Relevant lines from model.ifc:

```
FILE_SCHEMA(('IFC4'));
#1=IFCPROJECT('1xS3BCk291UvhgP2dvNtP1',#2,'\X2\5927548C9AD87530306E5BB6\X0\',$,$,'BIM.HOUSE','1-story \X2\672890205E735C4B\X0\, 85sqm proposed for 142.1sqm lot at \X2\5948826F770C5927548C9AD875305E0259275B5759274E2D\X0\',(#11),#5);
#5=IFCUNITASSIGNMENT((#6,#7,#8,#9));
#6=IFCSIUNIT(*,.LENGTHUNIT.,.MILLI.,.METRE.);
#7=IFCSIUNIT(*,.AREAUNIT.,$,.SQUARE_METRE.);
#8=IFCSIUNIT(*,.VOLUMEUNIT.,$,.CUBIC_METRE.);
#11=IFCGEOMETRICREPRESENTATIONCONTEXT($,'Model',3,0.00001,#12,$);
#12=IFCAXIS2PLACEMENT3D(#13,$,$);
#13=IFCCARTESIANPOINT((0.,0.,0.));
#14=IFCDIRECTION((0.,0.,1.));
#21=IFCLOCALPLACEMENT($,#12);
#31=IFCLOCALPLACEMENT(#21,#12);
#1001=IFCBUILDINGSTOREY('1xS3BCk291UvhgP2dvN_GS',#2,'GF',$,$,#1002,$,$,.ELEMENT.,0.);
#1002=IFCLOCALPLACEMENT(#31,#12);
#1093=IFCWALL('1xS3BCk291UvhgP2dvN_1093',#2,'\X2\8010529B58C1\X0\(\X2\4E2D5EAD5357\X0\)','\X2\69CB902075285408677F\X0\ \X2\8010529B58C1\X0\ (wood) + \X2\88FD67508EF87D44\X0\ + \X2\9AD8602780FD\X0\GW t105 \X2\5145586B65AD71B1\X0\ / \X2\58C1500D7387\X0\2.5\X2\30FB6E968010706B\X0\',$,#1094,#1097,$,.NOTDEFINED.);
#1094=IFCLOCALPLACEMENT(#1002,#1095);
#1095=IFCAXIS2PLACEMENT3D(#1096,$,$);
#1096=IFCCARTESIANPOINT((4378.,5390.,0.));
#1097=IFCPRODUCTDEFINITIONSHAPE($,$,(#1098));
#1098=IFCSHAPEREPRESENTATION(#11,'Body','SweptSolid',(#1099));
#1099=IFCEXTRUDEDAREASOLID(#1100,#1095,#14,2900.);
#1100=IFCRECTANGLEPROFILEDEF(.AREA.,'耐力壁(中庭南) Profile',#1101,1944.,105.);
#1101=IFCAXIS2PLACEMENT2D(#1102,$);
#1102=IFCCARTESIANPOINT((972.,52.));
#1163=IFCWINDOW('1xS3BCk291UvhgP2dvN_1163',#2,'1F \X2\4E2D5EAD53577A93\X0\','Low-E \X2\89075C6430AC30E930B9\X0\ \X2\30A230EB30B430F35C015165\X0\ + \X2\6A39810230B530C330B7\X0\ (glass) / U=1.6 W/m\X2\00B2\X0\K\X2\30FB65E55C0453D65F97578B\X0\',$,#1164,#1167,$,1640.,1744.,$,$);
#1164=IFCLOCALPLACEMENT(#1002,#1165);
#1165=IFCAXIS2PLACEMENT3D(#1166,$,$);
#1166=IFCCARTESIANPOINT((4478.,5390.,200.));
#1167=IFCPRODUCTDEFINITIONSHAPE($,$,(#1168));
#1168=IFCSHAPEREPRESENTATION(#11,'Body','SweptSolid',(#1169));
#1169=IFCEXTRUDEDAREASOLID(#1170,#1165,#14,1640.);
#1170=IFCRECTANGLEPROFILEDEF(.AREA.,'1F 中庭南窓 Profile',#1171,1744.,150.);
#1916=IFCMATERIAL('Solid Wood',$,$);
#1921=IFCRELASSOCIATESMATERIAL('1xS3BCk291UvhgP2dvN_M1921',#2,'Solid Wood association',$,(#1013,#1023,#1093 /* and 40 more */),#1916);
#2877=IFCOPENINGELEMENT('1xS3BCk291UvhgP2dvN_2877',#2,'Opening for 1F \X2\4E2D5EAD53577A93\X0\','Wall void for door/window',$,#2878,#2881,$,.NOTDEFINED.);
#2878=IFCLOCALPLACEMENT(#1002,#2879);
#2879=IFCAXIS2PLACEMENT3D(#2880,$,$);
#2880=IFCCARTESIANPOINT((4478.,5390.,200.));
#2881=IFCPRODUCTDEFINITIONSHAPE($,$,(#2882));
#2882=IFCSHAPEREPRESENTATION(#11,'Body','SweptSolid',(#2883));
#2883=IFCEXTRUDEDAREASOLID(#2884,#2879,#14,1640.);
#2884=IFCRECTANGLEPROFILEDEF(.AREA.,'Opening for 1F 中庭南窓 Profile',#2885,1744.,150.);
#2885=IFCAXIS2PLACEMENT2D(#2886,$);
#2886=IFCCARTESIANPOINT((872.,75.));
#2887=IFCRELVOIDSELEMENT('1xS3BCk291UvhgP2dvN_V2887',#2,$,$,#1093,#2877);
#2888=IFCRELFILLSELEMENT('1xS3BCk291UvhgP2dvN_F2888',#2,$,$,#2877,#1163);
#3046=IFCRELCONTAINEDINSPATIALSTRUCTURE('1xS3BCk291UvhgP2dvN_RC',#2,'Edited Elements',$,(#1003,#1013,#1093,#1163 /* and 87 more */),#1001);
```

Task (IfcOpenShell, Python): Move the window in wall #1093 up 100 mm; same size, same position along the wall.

```python
import numpy as np
import ifcopenshell
import ifcopenshell.api.geometry
import ifcopenshell.util.placement
import ifcopenshell.util.unit

model = ifcopenshell.open("model.ifc")
unit_scale = ifcopenshell.util.unit.calculate_unit_scale(model)

window = model.by_id(1163)
opening = window.FillsVoids[0].RelatingOpeningElement
dz = 100.0

shift = np.array([0.0, 0.0, dz])
# The window is not placed relative to its opening, so move both.
for product in (opening, window):
    matrix = ifcopenshell.util.placement.get_local_placement(product.ObjectPlacement)
    matrix[:3, 3] += shift
    ifcopenshell.api.geometry.edit_object_placement(model, product=product, matrix=matrix, is_si=False)

print(f"moved by {dz * unit_scale:+.3f} m")

model.write("model_edited.ifc")
```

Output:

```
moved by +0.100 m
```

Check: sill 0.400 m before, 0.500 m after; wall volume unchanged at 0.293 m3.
